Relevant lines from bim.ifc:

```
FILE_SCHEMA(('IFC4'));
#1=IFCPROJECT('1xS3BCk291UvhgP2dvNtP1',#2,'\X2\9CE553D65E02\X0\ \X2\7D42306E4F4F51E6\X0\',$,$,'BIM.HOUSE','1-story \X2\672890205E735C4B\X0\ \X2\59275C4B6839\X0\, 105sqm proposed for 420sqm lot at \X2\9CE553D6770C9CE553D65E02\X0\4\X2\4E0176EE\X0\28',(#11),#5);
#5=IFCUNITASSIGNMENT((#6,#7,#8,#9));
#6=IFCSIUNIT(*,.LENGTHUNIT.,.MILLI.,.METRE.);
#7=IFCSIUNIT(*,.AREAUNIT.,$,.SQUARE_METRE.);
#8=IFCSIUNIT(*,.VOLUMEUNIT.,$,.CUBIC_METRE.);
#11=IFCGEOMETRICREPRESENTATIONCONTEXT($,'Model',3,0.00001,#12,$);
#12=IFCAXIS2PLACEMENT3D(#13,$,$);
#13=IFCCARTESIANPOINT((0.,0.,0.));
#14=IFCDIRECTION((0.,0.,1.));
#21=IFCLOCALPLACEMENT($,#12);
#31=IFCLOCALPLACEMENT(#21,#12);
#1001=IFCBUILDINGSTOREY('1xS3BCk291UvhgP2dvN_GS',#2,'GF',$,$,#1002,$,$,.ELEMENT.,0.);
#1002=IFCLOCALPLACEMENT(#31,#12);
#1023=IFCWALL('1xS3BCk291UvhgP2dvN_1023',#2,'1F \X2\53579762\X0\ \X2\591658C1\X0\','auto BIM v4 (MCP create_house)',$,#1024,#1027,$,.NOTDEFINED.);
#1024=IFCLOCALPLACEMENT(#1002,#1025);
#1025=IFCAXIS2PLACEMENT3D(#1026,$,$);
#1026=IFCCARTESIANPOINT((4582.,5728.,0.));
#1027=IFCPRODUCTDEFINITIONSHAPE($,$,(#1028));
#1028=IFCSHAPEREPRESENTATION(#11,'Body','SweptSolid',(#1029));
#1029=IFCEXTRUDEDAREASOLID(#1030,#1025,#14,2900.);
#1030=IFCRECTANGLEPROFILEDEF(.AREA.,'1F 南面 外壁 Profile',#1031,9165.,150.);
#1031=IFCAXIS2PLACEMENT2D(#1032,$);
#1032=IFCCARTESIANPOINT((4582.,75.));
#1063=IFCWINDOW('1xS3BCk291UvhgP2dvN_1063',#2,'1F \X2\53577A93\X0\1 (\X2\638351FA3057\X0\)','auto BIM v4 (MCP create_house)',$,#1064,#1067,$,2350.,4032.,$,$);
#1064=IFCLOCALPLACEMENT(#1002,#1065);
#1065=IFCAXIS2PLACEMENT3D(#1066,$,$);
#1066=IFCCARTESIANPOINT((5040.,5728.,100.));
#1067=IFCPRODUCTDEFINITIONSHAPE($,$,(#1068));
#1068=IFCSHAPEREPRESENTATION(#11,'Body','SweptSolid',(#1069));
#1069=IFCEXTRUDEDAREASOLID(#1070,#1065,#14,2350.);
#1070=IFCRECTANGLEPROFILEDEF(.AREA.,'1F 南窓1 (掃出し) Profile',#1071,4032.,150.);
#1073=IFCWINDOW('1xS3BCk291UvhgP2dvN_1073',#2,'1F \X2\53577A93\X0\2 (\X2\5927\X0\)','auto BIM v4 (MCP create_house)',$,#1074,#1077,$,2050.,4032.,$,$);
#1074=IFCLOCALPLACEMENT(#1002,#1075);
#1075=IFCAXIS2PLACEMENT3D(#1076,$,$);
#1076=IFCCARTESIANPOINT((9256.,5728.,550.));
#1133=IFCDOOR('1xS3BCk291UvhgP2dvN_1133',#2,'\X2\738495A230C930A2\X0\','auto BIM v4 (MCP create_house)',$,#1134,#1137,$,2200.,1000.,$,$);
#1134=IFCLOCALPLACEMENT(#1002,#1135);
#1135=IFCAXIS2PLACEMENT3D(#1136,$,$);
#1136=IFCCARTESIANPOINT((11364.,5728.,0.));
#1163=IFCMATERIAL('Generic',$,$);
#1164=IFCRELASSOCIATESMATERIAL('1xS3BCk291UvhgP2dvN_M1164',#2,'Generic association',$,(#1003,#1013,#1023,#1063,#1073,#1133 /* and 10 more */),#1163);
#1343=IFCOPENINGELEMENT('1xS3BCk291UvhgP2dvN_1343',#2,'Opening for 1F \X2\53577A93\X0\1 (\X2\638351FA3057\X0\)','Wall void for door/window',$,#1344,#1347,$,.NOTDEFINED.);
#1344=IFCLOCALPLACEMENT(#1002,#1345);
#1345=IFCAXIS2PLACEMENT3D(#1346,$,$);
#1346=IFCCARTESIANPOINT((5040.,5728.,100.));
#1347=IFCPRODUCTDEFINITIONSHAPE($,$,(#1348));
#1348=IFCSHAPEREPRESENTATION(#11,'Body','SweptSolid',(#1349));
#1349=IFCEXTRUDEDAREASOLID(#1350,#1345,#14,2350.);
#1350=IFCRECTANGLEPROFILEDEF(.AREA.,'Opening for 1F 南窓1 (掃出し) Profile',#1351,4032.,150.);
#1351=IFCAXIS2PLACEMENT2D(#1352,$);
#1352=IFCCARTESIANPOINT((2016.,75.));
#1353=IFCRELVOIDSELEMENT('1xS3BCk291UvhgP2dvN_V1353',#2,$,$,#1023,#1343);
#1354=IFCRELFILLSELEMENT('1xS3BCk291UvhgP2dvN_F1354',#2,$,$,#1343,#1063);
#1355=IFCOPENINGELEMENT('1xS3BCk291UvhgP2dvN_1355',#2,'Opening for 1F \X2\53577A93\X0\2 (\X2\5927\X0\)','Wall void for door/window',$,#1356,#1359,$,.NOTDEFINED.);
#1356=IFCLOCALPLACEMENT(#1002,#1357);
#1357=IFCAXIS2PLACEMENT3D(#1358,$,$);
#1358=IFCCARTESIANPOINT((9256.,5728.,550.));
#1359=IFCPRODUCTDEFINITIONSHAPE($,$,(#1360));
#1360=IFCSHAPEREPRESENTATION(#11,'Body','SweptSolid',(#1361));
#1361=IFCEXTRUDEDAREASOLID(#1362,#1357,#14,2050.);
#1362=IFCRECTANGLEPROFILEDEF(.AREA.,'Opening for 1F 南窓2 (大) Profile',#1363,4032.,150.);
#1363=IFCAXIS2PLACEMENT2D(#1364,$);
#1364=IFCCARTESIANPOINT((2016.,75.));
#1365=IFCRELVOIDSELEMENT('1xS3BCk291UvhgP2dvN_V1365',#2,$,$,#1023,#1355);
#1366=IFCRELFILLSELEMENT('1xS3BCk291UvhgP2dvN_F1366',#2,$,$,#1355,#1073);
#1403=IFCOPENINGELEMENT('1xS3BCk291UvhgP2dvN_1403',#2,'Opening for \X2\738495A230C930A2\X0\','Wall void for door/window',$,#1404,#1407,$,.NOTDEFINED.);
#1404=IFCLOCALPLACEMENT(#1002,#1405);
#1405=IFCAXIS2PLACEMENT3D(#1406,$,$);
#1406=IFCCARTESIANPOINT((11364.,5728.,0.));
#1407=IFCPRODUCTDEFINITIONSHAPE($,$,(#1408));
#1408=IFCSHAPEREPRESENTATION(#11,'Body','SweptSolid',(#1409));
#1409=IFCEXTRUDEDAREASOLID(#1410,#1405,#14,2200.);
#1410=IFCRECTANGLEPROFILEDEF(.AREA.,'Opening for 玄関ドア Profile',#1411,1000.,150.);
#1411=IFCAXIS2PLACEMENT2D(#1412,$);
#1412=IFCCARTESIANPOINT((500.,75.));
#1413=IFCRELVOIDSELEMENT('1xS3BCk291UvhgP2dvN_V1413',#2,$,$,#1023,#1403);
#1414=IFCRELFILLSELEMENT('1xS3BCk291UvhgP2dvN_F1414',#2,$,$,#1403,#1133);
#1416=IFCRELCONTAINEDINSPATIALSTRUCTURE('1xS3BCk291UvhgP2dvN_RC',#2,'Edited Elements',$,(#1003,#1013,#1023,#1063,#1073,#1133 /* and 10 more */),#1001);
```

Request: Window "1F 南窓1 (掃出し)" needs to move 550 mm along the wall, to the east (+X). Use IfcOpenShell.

```python
import ifcopenshell
import ifcopenshell.api.geometry
import ifcopenshell.util.placement

model = ifcopenshell.open("bim.ifc")

window = model.by_guid("1xS3BCk291UvhgP2dvN_1063")
opening = window.FillsVoids[0].RelatingOpeningElement
wall = opening.VoidsElements[0].RelatingBuildingElement

wall_matrix = ifcopenshell.util.placement.get_local_placement(wall.ObjectPlacement)
shift = wall_matrix[:3, 0] * 550.0
before = ifcopenshell.util.placement.get_local_placement(window.ObjectPlacement)[:3, 3].copy()

# The window is not placed relative to its opening, so move both.
for product in (opening, window):
    matrix = ifcopenshell.util.placement.get_local_placement(product.ObjectPlacement)
    matrix[:3, 3] += shift
    ifcopenshell.api.geometry.edit_object_placement(model, product=product, matrix=matrix, is_si=False)

after = ifcopenshell.util.placement.get_local_placement(window.ObjectPlacement)[:3, 3]
print("window moved by", (after - before).round(3) + 0.0)

model.write("bim_updated.ifc")
```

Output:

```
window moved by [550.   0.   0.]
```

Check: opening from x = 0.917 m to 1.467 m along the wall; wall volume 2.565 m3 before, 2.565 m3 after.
